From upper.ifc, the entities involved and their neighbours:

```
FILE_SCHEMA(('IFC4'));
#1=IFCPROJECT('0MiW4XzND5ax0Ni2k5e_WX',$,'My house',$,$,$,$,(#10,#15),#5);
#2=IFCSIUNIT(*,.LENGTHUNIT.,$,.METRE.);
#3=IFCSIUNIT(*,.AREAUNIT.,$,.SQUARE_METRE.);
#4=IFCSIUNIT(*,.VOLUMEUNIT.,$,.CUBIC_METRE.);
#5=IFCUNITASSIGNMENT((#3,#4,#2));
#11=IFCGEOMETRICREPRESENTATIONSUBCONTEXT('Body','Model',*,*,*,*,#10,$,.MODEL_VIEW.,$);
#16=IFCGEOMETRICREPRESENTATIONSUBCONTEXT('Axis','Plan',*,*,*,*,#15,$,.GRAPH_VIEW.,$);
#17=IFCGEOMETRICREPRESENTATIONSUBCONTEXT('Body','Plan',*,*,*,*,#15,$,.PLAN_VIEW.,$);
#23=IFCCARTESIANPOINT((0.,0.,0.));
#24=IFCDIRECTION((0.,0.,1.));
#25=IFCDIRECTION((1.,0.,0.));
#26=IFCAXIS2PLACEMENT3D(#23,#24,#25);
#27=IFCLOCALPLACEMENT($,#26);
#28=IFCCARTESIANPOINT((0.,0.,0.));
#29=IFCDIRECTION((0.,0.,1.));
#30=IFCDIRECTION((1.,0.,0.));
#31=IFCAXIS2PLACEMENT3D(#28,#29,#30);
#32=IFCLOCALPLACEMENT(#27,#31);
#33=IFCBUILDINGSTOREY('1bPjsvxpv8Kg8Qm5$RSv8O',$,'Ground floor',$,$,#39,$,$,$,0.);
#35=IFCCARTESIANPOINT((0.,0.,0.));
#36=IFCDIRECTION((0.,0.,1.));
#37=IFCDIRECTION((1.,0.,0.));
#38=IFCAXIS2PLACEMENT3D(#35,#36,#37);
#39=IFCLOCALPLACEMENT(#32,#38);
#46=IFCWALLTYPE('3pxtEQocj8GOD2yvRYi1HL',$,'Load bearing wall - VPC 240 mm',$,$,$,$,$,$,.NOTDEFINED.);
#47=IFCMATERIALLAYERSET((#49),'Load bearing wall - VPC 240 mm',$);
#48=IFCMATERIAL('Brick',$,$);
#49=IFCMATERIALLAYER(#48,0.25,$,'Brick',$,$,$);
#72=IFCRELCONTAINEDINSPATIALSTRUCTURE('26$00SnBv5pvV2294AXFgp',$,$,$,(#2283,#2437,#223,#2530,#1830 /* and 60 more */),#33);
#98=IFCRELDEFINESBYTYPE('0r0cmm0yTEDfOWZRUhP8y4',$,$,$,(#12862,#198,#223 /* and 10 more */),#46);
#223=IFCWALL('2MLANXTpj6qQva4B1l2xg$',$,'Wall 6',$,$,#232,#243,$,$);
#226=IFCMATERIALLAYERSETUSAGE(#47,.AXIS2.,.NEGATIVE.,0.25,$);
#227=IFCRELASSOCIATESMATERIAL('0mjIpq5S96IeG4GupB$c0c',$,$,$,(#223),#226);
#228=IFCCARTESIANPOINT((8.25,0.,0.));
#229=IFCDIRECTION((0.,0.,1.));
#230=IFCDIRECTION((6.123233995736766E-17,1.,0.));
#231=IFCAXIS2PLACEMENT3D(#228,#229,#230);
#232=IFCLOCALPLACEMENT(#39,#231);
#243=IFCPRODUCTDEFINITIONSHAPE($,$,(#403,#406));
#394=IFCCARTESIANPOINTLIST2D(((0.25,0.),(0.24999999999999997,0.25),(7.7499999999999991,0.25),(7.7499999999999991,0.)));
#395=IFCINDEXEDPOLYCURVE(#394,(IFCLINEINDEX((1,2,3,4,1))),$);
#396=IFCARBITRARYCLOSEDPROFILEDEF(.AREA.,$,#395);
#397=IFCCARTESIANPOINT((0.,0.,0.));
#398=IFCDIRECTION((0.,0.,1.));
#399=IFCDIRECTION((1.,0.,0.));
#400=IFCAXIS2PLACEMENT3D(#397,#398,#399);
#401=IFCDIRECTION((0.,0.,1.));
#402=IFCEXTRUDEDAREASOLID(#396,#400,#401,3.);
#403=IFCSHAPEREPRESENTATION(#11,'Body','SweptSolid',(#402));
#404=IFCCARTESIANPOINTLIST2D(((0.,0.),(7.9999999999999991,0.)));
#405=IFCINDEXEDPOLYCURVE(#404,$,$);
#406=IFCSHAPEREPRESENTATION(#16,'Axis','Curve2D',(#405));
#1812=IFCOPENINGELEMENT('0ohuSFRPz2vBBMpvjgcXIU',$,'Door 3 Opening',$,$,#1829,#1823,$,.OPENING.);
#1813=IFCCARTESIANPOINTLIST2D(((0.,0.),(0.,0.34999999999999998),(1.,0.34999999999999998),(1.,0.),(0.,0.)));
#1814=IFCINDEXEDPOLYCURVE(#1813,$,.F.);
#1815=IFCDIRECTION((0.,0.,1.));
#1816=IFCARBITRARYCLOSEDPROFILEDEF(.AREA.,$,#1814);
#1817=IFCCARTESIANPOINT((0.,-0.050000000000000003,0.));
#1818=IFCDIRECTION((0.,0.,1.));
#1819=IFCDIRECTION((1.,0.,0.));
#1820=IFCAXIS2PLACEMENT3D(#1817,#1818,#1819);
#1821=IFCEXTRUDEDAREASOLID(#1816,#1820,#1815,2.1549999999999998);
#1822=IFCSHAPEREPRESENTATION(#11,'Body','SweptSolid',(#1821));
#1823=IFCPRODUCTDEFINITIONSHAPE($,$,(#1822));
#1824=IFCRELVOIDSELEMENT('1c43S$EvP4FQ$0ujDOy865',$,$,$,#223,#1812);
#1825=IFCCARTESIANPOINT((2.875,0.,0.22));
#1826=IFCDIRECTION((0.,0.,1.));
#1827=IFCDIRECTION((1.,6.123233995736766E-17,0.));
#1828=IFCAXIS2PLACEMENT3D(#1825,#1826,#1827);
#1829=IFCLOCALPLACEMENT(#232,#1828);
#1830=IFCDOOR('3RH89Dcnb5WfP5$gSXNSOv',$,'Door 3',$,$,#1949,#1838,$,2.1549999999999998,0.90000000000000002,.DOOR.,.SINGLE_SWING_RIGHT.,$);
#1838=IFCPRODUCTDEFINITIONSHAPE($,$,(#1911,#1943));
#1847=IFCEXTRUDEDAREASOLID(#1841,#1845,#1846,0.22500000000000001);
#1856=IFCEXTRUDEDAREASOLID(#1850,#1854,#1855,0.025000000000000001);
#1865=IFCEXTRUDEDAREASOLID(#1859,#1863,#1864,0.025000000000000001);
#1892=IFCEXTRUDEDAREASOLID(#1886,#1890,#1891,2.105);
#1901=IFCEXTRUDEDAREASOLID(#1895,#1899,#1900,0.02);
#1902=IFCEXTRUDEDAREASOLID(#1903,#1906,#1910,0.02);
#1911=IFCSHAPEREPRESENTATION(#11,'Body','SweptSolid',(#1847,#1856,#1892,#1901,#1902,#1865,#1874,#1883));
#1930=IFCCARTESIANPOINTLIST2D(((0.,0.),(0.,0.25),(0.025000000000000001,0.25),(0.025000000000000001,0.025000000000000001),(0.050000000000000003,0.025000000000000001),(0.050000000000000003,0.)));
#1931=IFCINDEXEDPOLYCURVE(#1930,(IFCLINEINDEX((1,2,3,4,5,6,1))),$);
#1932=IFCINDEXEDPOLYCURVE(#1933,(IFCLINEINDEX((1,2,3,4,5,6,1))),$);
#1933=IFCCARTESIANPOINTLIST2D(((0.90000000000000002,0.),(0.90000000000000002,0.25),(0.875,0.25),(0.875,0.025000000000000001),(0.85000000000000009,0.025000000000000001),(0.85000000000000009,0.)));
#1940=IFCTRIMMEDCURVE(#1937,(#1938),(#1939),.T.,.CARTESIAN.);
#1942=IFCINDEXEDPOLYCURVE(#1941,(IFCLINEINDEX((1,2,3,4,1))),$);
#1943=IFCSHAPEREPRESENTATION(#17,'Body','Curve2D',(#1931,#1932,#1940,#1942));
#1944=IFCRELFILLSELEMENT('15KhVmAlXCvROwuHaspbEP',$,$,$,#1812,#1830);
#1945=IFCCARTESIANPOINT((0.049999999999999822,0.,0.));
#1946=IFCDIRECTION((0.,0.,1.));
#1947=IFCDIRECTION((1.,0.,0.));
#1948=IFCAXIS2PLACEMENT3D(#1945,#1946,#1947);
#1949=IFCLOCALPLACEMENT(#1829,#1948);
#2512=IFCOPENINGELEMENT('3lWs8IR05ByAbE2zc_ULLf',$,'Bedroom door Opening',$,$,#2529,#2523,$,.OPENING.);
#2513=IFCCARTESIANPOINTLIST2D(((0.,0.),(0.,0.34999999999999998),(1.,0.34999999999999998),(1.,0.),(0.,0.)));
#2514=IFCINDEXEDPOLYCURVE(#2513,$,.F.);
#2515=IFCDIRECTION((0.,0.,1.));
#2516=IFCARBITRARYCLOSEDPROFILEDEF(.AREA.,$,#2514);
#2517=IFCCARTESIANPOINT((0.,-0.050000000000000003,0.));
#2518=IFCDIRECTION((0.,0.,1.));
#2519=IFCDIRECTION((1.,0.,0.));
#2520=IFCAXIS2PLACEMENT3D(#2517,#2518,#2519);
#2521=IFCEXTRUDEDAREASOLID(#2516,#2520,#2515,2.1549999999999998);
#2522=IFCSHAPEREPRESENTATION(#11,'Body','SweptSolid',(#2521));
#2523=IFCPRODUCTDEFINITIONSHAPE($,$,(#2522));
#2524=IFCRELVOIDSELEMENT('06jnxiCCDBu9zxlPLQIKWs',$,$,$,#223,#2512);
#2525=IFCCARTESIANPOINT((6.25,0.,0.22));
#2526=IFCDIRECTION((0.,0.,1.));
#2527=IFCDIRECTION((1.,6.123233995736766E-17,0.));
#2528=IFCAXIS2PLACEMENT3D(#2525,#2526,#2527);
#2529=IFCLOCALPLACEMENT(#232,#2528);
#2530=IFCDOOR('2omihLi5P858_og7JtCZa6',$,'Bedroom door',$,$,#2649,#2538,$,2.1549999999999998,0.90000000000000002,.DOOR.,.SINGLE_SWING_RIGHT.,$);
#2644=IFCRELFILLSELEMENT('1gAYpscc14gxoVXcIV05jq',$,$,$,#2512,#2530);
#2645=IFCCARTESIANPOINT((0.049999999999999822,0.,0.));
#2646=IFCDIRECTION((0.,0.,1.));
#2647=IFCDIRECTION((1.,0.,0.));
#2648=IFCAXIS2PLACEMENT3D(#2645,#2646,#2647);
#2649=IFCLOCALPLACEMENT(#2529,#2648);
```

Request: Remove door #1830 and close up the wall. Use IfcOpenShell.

```python
import ifcopenshell
import ifcopenshell.api.feature
import ifcopenshell.api.root
import ifcopenshell.geom
import ifcopenshell.util.shape

model = ifcopenshell.open("upper.ifc")
settings = ifcopenshell.geom.settings()


def volume(element):
    """Net volume in cubic metres, openings subtracted."""
    shape = ifcopenshell.geom.create_shape(settings, element)
    return ifcopenshell.util.shape.get_volume(shape.geometry)


door = model.by_id(1830)
opening = door.FillsVoids[0].RelatingOpeningElement
wall = opening.VoidsElements[0].RelatingBuildingElement
before = volume(wall)

ifcopenshell.api.root.remove_product(model, product=door)
ifcopenshell.api.feature.remove_feature(model, feature=opening)

after = volume(wall)

print(f"wall volume {before:.3f} -> {after:.3f} m3")

model.write("upper-out.ifc")
```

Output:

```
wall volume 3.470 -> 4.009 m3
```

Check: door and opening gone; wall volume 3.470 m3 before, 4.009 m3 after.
